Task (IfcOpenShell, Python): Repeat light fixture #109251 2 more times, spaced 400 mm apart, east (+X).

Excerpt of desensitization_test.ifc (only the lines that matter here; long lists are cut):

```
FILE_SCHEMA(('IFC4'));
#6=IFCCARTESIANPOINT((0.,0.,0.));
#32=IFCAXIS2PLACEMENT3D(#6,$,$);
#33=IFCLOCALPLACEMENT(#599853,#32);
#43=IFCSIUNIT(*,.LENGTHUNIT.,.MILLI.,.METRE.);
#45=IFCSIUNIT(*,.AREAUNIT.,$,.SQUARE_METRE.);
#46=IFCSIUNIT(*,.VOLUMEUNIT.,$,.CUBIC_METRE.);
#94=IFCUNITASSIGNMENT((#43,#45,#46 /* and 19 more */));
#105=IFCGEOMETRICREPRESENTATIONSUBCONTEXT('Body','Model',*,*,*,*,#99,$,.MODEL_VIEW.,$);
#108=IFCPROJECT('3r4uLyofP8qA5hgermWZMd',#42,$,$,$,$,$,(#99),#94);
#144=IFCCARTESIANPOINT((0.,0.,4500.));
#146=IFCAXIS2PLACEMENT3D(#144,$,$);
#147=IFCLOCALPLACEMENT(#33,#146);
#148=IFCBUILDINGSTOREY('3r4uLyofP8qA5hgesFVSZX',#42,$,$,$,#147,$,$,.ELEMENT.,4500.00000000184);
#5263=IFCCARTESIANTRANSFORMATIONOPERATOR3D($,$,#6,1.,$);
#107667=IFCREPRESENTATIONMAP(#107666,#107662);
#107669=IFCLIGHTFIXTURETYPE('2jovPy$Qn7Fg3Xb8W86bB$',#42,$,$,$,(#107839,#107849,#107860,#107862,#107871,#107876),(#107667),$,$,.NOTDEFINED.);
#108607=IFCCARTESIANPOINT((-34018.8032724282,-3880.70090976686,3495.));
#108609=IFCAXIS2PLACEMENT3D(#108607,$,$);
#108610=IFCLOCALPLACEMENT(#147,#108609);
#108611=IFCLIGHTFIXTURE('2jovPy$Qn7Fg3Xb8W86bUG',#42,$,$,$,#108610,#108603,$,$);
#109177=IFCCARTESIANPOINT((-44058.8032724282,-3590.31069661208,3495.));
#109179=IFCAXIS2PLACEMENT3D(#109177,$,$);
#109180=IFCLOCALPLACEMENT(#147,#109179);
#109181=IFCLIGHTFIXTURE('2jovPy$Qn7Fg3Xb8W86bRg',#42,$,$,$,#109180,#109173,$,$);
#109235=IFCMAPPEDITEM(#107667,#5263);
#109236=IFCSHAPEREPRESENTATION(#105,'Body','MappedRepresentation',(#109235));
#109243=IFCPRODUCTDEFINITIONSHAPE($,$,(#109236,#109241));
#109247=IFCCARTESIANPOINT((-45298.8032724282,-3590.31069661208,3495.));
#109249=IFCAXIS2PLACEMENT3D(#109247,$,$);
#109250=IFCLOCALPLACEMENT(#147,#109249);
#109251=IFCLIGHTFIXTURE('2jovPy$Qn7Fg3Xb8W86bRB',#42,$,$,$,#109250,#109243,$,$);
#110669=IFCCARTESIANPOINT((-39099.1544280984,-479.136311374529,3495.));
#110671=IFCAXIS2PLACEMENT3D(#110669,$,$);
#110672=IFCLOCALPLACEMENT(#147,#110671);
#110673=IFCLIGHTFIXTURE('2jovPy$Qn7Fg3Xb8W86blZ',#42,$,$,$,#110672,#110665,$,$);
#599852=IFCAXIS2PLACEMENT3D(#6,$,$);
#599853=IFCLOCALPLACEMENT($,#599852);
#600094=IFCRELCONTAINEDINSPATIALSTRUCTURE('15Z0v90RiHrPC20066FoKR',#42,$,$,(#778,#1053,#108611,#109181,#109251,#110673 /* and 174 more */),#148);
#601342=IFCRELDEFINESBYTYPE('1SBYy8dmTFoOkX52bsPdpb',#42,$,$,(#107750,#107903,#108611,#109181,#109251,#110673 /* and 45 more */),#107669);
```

```python
import numpy as np
import ifcopenshell
import ifcopenshell.api.geometry
import ifcopenshell.api.root
import ifcopenshell.util.element
import ifcopenshell.util.placement
import ifcopenshell.util.unit

model = ifcopenshell.open("desensitization_test.ifc")
unit_scale = ifcopenshell.util.unit.calculate_unit_scale(model)


def reuse_history(source, copy):
    """copy_class also copies each property set's owner history, people and application; keep the originals."""
    for rel in copy.IsDefinedBy:
        if rel.is_a("IfcRelDefinesByProperties") and (history := rel.RelatingPropertyDefinition.OwnerHistory):
            rel.RelatingPropertyDefinition.OwnerHistory = source.OwnerHistory
            ifcopenshell.util.element.remove_deep2(model, history)


source = model.by_guid("2jovPy$Qn7Fg3Xb8W86bRB")
base = ifcopenshell.util.placement.get_local_placement(source.ObjectPlacement)
step = np.array([1.0, 0.0, 0.0]) * 0.4 / unit_scale

for i in range(1, 3):
    copy = ifcopenshell.api.root.copy_class(model, product=source)
    copy.Representation = ifcopenshell.util.element.copy_deep(
        model, source.Representation, exclude=["IfcGeometricRepresentationContext", "IfcRepresentationMap"]
    )
    reuse_history(source, copy)
    matrix = base.copy()
    matrix[:3, 3] += i * step
    print("added at", matrix[:3, 3].round(3) + 0.0)
    ifcopenshell.api.geometry.edit_object_placement(model, product=copy, matrix=matrix, is_si=False)

model.write("desensitization_test_v2.ifc")
```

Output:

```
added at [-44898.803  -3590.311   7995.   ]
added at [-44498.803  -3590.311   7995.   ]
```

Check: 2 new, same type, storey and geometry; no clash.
